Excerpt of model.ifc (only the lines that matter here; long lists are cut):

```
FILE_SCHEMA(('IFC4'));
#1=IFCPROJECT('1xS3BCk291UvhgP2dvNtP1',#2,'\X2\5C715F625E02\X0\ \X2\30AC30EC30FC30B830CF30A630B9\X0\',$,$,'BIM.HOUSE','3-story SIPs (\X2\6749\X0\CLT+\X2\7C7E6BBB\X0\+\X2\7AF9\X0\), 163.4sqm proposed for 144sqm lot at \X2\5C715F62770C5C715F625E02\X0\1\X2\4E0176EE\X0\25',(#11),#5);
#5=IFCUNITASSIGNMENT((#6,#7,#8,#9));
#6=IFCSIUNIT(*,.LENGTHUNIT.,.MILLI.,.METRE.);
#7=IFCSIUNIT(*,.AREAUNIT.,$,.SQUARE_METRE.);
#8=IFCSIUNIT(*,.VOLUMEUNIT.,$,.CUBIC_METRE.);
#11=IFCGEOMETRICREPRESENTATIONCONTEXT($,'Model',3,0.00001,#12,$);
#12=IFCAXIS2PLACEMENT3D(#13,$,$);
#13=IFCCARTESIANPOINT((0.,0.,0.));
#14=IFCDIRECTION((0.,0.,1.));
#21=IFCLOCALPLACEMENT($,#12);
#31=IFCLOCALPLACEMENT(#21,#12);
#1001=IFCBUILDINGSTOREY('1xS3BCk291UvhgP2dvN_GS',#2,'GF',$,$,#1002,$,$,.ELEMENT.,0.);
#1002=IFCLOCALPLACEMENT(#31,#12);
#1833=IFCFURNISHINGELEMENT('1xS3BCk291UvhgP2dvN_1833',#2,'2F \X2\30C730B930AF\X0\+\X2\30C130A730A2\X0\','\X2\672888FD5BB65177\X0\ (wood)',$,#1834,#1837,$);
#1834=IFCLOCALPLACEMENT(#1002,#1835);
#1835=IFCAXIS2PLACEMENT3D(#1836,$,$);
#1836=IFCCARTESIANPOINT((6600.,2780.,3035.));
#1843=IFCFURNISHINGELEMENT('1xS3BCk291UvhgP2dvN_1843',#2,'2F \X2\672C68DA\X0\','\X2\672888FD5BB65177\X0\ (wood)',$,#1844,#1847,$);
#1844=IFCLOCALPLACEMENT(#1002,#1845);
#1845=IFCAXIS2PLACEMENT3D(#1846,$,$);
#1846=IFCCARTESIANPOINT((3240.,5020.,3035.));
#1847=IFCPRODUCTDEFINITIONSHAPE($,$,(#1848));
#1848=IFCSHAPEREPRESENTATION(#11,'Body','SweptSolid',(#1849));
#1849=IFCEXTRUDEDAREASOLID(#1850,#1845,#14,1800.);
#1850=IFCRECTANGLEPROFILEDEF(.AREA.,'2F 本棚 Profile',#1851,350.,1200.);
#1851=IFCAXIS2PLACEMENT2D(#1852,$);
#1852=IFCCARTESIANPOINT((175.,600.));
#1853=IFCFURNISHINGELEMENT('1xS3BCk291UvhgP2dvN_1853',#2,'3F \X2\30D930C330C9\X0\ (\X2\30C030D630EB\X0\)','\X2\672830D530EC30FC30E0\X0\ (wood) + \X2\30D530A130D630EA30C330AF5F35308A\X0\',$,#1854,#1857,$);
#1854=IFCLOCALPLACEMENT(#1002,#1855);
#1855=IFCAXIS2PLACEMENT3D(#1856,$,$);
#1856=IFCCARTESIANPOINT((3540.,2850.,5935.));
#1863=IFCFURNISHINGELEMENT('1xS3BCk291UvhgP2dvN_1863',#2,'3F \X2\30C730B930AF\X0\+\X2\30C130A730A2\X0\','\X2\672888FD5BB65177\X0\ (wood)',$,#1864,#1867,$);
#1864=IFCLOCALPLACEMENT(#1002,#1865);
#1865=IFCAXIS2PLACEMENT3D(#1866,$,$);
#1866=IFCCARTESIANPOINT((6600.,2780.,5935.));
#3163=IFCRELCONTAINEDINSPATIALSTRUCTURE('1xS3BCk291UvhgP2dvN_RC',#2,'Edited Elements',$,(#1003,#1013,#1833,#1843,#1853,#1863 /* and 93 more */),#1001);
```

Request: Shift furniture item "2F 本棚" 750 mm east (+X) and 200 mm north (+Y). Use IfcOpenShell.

```python
import ifcopenshell
import ifcopenshell.api.geometry
import ifcopenshell.util.placement
import ifcopenshell.util.unit

model = ifcopenshell.open("model.ifc")
unit_scale = ifcopenshell.util.unit.calculate_unit_scale(model)

item = model.by_guid("1xS3BCk291UvhgP2dvN_1843")
matrix = ifcopenshell.util.placement.get_local_placement(item.ObjectPlacement)
matrix[0, 3] += 0.75 / unit_scale
matrix[1, 3] += 0.2 / unit_scale
ifcopenshell.api.geometry.edit_object_placement(model, product=item, matrix=matrix, is_si=False)

print(ifcopenshell.util.placement.get_local_placement(item.ObjectPlacement).round(3) + 0.0)

model.write("model-out.ifc")
```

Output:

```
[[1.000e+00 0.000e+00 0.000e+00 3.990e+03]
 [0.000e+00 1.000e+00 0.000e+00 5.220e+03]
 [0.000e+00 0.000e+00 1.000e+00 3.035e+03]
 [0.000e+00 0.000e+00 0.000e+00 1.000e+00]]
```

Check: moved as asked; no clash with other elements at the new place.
